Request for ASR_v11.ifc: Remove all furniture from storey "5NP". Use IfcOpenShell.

First a look at what the model holds.

```python
import ifcopenshell
import ifcopenshell.util.element

model = ifcopenshell.open("ASR_v11.ifc")
print(model.schema)
storey = next(s for s in model.by_type("IfcBuildingStorey") if s.Name == "5NP")
furniture = [e for e in ifcopenshell.util.element.get_decomposition(storey) if e.is_a("IfcFurnishingElement")]
seen = {}
for e in furniture:
    element_type = ifcopenshell.util.element.get_type(e)
    name = element_type.Name if element_type not in (None, e) else None
    seen[name] = seen.get(name, 0) + 1
for name, count in sorted(seen.items(), key=str):
    print(count, "x", name)
```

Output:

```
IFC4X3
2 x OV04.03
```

```python
import ifcopenshell
import ifcopenshell.api.root
import ifcopenshell.util.element

model = ifcopenshell.open("ASR_v11.ifc")

storey = next(s for s in model.by_type("IfcBuildingStorey") if s.Name == "5NP")
furniture = [e for e in ifcopenshell.util.element.get_decomposition(storey) if e.is_a("IfcFurnishingElement")]

for e in furniture:
    ifcopenshell.api.root.remove_product(model, product=e)
print(len(furniture), "removed")

model.write("ASR_v11_v2.ifc")
```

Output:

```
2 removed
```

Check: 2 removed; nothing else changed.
